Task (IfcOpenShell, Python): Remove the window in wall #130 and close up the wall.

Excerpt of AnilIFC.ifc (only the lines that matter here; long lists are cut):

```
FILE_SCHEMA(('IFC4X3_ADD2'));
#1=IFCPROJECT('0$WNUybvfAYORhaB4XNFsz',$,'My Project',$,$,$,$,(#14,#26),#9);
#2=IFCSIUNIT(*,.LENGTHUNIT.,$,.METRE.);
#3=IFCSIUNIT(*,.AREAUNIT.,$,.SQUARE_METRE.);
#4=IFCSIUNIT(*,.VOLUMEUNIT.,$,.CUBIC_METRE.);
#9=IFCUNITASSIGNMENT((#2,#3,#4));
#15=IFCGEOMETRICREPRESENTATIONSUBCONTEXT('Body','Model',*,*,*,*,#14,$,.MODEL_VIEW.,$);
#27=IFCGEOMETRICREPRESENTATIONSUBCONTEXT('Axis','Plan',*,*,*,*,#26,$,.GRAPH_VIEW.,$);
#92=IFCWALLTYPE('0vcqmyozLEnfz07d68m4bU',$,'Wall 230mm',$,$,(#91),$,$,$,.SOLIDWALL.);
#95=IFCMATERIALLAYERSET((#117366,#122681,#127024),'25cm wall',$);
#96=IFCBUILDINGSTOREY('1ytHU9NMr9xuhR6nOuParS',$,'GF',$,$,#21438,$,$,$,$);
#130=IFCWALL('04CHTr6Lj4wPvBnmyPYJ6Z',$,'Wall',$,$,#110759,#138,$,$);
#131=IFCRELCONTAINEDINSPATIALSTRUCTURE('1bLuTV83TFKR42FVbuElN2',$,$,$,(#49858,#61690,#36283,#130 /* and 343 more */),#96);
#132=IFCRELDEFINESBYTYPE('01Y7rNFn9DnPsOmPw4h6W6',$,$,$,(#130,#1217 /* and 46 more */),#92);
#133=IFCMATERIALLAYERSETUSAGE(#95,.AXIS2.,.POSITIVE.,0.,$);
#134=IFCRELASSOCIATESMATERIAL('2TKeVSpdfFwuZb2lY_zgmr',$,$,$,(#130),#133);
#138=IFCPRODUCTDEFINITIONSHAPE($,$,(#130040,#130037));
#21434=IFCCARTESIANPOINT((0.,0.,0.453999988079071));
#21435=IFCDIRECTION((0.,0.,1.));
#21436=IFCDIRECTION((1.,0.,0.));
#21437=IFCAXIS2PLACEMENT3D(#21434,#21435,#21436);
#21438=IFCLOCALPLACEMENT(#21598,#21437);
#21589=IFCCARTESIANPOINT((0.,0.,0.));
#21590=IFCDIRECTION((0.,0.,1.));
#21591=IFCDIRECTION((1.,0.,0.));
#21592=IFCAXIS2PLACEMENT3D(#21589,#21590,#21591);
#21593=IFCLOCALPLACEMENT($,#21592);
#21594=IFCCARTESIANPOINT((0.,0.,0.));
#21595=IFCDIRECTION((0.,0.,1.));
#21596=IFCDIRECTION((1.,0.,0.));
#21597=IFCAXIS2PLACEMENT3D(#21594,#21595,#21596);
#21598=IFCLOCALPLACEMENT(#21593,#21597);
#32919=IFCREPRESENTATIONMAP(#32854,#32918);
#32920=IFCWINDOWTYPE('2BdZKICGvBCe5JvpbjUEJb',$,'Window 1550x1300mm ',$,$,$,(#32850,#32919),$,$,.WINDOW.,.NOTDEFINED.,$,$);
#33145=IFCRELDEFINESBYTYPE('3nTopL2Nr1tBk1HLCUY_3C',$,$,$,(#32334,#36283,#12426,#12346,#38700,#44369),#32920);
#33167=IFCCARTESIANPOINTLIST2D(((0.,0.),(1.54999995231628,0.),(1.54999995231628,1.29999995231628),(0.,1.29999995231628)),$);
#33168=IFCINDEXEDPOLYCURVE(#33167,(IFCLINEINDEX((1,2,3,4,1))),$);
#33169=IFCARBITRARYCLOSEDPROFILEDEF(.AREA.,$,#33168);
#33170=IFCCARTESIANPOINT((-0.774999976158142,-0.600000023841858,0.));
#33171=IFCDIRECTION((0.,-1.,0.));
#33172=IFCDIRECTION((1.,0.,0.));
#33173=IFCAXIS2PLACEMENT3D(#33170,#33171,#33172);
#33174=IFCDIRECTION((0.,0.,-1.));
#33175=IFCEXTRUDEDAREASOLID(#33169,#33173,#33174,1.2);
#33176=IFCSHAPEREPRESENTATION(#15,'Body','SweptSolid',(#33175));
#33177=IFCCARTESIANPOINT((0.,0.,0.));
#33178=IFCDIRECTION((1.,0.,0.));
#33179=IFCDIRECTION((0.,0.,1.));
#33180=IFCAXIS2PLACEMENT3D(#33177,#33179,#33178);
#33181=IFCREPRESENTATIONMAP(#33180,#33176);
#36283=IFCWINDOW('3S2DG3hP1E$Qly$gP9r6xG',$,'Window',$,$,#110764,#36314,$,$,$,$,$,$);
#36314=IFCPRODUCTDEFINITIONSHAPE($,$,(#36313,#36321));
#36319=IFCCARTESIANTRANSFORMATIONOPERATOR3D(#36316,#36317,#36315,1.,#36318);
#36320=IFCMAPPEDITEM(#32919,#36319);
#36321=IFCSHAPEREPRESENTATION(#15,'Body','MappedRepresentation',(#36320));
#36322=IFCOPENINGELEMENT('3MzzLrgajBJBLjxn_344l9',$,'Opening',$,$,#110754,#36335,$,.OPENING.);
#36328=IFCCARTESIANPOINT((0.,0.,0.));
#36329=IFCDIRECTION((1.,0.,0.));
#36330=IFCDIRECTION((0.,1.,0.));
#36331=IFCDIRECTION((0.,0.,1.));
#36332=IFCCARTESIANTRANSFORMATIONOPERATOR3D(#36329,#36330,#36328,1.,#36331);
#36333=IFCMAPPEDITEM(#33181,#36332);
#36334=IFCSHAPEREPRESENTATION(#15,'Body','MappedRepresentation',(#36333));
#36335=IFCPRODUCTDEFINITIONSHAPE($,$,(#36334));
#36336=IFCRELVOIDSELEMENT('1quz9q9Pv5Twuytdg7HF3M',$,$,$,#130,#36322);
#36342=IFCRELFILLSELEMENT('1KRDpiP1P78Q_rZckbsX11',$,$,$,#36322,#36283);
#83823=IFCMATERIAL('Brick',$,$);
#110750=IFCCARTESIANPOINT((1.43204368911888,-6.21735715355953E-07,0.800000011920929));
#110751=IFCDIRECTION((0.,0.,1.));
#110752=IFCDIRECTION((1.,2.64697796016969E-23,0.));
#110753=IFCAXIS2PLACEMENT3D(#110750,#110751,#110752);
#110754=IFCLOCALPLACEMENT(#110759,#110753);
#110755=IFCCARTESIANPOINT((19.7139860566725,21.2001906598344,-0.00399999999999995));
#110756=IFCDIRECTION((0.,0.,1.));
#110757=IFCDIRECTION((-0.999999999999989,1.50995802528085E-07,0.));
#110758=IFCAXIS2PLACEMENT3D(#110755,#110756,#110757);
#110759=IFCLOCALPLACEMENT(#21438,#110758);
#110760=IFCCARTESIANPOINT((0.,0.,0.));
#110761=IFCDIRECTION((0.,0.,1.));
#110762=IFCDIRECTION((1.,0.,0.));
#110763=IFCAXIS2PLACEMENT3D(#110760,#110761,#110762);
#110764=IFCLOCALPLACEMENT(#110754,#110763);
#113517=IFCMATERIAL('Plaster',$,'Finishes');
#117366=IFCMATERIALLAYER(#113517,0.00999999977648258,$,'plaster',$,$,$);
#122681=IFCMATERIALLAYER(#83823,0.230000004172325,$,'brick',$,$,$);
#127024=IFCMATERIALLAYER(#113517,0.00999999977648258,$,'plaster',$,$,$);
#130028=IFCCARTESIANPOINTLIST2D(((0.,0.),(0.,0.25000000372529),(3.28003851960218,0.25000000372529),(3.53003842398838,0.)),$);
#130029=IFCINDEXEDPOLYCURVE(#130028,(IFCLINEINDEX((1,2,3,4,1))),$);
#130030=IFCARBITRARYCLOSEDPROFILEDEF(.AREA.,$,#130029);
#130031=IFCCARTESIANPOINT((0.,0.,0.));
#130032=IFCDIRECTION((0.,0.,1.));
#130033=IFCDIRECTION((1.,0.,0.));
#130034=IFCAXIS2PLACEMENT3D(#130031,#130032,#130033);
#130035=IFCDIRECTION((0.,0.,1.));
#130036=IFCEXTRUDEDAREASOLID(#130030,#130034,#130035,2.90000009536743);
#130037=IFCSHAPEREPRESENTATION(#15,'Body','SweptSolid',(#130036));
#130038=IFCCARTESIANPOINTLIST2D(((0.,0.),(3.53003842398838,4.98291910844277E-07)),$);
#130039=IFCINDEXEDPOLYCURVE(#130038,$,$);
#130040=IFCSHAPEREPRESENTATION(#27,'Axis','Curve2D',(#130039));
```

```python
import ifcopenshell
import ifcopenshell.api.feature
import ifcopenshell.api.root
import ifcopenshell.geom
import ifcopenshell.util.shape

model = ifcopenshell.open("AnilIFC.ifc")
settings = ifcopenshell.geom.settings()


def volume(element):
    """Net volume in cubic metres, openings subtracted."""
    shape = ifcopenshell.geom.create_shape(settings, element)
    return ifcopenshell.util.shape.get_volume(shape.geometry)


window = model.by_id(36283)
opening = window.FillsVoids[0].RelatingOpeningElement
wall = opening.VoidsElements[0].RelatingBuildingElement
before = volume(wall)

ifcopenshell.api.root.remove_product(model, product=window)
ifcopenshell.api.feature.remove_feature(model, feature=opening)

after = volume(wall)

print(f"wall volume {before:.3f} -> {after:.3f} m3")

model.write("AnilIFC_rev.ifc")
```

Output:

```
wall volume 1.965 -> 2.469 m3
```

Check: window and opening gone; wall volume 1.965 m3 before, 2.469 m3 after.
